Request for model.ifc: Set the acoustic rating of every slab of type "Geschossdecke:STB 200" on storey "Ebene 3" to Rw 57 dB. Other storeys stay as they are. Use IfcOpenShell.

First a look at what the model holds.

```python
import ifcopenshell
import ifcopenshell.util.element

model = ifcopenshell.open("model.ifc")
print(model.schema)
storey = next(s for s in model.by_type("IfcBuildingStorey") if s.Name == "Ebene 3")
slabs = [e for e in ifcopenshell.util.element.get_decomposition(storey) if e.is_a("IfcSlab")]
seen = {}
for e in slabs:
    element_type = ifcopenshell.util.element.get_type(e)
    key = (element_type.Name if element_type != e and element_type else None, ifcopenshell.util.element.get_pset(e, "Pset_SlabCommon", "AcousticRating"))
    seen[key] = seen.get(key, 0) + 1
for (name, value), count in sorted(seen.items(), key=str):
    print(count, "x", name, "|", value)
```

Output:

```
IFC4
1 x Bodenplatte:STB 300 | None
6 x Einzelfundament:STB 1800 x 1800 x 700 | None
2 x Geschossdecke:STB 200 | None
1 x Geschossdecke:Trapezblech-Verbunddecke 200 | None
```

```python
import ifcopenshell
import ifcopenshell.api.pset
import ifcopenshell.util.element

model = ifcopenshell.open("model.ifc")

storey = next(s for s in model.by_type("IfcBuildingStorey") if s.Name == "Ebene 3")
slabs = [e for e in ifcopenshell.util.element.get_decomposition(storey) if e.is_a("IfcSlab")]

count = 0
for e in slabs:
    element_type = ifcopenshell.util.element.get_type(e)
    if element_type in (None, e) or element_type.Name != "Geschossdecke:STB 200":
        continue
    # add_pset returns the element's existing set when there is one.
    pset = ifcopenshell.api.pset.add_pset(model, product=e, name="Pset_SlabCommon")
    ifcopenshell.api.pset.edit_pset(model, pset=pset, properties={"AcousticRating": "Rw 57 dB"})
    count += 1

print(count, "slabs updated")

model.write("model_v2.ifc")
```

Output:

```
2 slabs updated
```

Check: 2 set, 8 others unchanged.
